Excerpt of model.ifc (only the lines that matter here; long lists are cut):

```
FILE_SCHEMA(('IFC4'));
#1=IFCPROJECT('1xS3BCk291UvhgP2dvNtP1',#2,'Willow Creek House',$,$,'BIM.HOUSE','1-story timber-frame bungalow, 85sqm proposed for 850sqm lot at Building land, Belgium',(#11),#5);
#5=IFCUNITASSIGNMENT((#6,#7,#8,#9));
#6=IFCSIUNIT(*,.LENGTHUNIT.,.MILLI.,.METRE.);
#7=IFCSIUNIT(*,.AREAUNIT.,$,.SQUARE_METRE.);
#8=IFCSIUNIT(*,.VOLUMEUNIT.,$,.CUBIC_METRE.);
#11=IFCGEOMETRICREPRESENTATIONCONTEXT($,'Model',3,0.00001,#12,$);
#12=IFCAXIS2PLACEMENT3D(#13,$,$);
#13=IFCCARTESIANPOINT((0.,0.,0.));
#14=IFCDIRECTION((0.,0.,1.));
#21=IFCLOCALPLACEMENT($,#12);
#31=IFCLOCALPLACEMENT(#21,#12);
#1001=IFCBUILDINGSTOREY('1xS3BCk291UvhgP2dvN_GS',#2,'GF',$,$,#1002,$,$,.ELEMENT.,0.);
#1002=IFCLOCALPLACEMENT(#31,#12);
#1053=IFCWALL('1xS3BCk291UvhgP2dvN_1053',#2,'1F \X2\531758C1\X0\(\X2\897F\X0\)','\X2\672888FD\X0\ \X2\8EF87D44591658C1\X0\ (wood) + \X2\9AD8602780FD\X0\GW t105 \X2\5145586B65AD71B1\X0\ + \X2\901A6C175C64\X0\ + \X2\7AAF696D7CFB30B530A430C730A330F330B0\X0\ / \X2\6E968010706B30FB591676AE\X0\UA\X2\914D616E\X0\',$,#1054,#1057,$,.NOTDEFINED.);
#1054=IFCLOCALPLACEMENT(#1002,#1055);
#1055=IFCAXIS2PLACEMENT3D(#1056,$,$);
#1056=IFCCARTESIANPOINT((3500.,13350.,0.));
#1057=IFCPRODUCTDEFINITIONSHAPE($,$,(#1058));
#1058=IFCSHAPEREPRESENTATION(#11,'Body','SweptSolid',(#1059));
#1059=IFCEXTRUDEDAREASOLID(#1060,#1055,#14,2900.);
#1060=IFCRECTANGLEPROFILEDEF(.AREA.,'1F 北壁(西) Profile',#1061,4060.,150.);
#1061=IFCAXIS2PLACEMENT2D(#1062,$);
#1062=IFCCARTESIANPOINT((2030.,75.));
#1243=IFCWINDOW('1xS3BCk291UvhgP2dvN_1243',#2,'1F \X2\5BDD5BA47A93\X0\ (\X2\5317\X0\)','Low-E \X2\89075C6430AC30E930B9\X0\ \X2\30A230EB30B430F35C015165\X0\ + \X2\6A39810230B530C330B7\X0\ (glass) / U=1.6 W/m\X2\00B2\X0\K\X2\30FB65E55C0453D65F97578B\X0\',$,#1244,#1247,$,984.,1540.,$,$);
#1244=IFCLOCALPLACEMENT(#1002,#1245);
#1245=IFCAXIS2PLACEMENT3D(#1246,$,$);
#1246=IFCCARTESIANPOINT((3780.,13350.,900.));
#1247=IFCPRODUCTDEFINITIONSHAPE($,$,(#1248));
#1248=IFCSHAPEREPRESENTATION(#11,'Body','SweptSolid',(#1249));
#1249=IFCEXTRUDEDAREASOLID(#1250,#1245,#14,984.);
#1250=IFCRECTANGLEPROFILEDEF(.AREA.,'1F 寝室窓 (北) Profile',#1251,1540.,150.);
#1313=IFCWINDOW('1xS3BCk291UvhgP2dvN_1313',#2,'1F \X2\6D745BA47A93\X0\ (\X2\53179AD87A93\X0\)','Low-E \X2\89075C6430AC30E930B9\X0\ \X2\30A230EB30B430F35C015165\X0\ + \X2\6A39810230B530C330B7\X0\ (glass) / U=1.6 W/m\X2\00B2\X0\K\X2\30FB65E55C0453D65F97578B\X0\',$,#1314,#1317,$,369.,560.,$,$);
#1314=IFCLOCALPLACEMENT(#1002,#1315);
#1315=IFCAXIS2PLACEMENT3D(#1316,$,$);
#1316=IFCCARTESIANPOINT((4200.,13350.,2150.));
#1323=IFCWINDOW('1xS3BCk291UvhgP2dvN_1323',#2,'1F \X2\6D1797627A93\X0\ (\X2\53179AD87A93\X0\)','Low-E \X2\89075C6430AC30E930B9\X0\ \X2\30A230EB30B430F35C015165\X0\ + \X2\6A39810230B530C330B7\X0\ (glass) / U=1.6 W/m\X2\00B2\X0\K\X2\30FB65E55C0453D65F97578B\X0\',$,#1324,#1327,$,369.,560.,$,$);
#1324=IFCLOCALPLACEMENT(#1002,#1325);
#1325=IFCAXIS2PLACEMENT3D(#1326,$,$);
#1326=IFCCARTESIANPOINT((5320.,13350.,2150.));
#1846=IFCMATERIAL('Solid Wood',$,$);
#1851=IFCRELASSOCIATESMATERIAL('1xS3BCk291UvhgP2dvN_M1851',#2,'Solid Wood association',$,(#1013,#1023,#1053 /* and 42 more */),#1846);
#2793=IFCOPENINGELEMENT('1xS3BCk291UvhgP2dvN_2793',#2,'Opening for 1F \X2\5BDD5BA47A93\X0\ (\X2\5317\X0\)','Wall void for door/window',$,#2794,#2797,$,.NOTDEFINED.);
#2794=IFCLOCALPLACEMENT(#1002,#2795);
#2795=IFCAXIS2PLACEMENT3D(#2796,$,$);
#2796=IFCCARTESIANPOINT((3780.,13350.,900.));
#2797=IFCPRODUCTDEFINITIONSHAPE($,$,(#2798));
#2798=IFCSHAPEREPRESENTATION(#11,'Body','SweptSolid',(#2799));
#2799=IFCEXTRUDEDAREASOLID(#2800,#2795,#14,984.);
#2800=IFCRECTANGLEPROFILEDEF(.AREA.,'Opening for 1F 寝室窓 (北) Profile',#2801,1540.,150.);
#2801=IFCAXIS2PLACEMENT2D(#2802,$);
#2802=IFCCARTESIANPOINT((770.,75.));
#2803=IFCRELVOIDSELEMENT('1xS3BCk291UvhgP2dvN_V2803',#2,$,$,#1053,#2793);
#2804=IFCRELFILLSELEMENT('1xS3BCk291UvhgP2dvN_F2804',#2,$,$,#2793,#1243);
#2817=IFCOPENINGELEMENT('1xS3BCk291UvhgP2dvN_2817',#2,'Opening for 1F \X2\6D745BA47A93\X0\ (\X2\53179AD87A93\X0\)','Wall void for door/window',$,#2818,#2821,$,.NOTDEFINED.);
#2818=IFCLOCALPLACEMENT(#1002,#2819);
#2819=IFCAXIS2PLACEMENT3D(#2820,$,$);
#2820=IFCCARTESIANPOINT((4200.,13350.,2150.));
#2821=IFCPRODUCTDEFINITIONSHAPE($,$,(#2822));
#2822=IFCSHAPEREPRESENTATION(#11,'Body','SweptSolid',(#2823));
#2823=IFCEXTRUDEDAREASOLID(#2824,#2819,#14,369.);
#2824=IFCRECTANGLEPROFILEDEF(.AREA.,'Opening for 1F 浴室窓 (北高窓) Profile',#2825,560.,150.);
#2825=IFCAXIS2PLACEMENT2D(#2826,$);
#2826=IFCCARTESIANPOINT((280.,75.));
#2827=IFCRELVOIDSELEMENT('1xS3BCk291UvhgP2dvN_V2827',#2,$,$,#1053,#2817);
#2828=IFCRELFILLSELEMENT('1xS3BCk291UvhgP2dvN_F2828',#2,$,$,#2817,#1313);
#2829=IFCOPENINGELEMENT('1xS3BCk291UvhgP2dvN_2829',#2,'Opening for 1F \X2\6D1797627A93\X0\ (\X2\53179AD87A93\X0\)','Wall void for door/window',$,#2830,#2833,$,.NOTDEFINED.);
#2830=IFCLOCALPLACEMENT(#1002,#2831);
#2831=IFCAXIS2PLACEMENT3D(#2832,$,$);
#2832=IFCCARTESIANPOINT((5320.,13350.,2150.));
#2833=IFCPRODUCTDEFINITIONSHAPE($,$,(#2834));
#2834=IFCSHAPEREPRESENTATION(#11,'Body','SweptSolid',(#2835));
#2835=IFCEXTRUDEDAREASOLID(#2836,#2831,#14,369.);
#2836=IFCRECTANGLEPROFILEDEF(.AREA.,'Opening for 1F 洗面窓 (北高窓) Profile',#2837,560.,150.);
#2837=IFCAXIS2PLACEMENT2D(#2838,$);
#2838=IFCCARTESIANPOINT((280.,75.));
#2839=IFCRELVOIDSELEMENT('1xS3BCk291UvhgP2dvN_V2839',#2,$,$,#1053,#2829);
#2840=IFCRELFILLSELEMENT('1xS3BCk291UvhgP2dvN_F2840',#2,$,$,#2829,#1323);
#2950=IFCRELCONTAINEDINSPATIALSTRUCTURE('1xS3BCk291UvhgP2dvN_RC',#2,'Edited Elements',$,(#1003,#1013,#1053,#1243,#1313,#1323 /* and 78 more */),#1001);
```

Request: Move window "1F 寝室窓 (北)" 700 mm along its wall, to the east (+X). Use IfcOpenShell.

```python
import ifcopenshell
import ifcopenshell.api.geometry
import ifcopenshell.util.placement

model = ifcopenshell.open("model.ifc")

window = model.by_guid("1xS3BCk291UvhgP2dvN_1243")
opening = window.FillsVoids[0].RelatingOpeningElement
wall = opening.VoidsElements[0].RelatingBuildingElement

wall_matrix = ifcopenshell.util.placement.get_local_placement(wall.ObjectPlacement)
shift = wall_matrix[:3, 0] * 700.0
before = ifcopenshell.util.placement.get_local_placement(window.ObjectPlacement)[:3, 3].copy()

# The window is not placed relative to its opening, so move both.
for product in (opening, window):
    matrix = ifcopenshell.util.placement.get_local_placement(product.ObjectPlacement)
    matrix[:3, 3] += shift
    ifcopenshell.api.geometry.edit_object_placement(model, product=product, matrix=matrix, is_si=False)

after = ifcopenshell.util.placement.get_local_placement(window.ObjectPlacement)[:3, 3]
print("window moved by", (after - before).round(3) + 0.0)

model.write("model_v2.ifc")
```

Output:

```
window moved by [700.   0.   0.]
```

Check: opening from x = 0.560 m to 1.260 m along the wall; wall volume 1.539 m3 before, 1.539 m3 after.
